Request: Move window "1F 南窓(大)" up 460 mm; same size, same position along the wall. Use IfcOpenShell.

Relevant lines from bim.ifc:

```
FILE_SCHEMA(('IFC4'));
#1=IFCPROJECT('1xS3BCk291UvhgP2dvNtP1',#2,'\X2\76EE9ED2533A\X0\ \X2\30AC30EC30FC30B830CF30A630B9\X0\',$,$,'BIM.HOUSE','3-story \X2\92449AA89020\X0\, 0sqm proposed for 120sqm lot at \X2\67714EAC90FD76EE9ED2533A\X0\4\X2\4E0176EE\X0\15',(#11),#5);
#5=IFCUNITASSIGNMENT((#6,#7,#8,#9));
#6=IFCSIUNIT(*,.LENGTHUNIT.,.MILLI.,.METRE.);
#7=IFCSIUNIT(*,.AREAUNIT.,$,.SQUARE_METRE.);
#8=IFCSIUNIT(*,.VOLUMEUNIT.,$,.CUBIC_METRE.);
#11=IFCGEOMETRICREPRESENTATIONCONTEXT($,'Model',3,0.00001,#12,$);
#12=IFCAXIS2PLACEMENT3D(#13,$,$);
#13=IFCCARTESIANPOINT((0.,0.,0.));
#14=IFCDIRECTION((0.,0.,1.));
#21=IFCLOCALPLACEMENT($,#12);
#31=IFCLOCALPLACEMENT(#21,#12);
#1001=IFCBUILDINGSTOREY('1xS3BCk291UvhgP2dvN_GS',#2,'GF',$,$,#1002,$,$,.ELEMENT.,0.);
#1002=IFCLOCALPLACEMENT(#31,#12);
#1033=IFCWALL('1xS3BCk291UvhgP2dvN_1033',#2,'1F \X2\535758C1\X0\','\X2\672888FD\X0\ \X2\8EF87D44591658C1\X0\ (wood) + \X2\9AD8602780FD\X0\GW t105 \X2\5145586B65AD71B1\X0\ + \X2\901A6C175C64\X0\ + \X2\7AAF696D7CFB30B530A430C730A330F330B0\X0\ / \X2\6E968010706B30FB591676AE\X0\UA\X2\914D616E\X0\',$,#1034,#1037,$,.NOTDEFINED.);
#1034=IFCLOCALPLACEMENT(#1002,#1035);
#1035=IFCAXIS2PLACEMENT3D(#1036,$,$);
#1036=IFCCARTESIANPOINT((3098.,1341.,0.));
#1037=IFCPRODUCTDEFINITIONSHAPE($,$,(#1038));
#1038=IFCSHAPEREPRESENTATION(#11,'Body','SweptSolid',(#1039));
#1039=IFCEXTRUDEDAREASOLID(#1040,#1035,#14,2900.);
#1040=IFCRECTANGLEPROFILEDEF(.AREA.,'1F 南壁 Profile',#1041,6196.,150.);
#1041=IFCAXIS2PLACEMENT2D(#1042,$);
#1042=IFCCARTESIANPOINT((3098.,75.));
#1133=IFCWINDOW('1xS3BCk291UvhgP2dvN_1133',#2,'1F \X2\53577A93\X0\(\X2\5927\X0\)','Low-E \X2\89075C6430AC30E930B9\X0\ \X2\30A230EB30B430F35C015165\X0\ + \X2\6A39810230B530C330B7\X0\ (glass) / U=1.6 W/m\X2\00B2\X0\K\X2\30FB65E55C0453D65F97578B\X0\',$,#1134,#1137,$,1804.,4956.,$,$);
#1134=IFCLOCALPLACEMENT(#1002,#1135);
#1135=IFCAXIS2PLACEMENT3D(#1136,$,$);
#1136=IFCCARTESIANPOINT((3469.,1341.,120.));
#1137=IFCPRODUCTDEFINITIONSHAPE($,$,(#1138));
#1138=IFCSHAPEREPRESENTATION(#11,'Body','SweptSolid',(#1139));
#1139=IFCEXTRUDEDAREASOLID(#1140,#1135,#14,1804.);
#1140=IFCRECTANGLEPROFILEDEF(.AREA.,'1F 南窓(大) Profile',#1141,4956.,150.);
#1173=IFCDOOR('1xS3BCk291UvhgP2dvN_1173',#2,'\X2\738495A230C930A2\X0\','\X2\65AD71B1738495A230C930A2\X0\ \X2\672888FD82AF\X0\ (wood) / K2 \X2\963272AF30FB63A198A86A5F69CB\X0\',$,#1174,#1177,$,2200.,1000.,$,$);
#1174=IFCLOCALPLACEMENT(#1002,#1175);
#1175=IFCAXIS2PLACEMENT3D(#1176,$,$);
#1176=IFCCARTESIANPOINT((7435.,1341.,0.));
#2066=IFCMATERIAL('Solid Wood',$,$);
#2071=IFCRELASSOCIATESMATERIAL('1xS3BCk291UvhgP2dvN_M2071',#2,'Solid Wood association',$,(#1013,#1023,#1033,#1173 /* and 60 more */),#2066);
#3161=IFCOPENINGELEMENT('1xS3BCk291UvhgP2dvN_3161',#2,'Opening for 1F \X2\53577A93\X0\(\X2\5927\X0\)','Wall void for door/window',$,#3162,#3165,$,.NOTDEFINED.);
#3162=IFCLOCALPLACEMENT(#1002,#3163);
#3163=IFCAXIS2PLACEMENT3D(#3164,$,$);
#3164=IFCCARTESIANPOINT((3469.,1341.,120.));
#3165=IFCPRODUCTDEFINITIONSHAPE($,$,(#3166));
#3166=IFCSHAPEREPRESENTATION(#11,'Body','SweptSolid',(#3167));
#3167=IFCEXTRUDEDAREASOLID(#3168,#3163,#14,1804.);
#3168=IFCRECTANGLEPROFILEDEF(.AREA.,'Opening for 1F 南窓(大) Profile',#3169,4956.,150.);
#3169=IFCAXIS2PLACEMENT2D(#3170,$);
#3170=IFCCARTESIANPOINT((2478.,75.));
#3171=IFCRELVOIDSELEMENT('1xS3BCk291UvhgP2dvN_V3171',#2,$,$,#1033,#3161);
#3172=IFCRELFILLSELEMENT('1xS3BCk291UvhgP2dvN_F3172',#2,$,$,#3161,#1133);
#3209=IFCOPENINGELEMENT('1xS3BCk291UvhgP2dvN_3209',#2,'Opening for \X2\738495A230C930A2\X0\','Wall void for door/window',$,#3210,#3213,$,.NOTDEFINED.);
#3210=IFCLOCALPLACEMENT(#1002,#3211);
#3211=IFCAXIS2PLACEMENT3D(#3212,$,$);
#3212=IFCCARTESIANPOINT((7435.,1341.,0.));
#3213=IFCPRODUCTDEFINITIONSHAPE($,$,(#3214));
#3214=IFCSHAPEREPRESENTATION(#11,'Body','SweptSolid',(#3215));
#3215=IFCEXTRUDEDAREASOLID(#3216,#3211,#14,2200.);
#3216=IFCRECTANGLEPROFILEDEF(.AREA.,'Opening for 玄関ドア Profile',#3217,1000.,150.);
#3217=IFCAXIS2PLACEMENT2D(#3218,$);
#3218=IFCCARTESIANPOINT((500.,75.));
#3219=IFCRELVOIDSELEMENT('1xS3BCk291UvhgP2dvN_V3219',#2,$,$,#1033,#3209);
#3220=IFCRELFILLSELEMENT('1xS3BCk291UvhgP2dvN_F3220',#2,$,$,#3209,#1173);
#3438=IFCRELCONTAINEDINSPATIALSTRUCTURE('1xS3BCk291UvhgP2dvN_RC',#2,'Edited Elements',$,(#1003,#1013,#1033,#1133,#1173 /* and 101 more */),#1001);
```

```python
import numpy as np
import ifcopenshell
import ifcopenshell.api.geometry
import ifcopenshell.util.placement
import ifcopenshell.util.unit

model = ifcopenshell.open("bim.ifc")
unit_scale = ifcopenshell.util.unit.calculate_unit_scale(model)

window = model.by_guid("1xS3BCk291UvhgP2dvN_1133")
opening = window.FillsVoids[0].RelatingOpeningElement
dz = 460.0

shift = np.array([0.0, 0.0, dz])
# The window is not placed relative to its opening, so move both.
for product in (opening, window):
    matrix = ifcopenshell.util.placement.get_local_placement(product.ObjectPlacement)
    matrix[:3, 3] += shift
    ifcopenshell.api.geometry.edit_object_placement(model, product=product, matrix=matrix, is_si=False)

print(f"moved by {dz * unit_scale:+.3f} m")

model.write("bim_rev.ifc")
```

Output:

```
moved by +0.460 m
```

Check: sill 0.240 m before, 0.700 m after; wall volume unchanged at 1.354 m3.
